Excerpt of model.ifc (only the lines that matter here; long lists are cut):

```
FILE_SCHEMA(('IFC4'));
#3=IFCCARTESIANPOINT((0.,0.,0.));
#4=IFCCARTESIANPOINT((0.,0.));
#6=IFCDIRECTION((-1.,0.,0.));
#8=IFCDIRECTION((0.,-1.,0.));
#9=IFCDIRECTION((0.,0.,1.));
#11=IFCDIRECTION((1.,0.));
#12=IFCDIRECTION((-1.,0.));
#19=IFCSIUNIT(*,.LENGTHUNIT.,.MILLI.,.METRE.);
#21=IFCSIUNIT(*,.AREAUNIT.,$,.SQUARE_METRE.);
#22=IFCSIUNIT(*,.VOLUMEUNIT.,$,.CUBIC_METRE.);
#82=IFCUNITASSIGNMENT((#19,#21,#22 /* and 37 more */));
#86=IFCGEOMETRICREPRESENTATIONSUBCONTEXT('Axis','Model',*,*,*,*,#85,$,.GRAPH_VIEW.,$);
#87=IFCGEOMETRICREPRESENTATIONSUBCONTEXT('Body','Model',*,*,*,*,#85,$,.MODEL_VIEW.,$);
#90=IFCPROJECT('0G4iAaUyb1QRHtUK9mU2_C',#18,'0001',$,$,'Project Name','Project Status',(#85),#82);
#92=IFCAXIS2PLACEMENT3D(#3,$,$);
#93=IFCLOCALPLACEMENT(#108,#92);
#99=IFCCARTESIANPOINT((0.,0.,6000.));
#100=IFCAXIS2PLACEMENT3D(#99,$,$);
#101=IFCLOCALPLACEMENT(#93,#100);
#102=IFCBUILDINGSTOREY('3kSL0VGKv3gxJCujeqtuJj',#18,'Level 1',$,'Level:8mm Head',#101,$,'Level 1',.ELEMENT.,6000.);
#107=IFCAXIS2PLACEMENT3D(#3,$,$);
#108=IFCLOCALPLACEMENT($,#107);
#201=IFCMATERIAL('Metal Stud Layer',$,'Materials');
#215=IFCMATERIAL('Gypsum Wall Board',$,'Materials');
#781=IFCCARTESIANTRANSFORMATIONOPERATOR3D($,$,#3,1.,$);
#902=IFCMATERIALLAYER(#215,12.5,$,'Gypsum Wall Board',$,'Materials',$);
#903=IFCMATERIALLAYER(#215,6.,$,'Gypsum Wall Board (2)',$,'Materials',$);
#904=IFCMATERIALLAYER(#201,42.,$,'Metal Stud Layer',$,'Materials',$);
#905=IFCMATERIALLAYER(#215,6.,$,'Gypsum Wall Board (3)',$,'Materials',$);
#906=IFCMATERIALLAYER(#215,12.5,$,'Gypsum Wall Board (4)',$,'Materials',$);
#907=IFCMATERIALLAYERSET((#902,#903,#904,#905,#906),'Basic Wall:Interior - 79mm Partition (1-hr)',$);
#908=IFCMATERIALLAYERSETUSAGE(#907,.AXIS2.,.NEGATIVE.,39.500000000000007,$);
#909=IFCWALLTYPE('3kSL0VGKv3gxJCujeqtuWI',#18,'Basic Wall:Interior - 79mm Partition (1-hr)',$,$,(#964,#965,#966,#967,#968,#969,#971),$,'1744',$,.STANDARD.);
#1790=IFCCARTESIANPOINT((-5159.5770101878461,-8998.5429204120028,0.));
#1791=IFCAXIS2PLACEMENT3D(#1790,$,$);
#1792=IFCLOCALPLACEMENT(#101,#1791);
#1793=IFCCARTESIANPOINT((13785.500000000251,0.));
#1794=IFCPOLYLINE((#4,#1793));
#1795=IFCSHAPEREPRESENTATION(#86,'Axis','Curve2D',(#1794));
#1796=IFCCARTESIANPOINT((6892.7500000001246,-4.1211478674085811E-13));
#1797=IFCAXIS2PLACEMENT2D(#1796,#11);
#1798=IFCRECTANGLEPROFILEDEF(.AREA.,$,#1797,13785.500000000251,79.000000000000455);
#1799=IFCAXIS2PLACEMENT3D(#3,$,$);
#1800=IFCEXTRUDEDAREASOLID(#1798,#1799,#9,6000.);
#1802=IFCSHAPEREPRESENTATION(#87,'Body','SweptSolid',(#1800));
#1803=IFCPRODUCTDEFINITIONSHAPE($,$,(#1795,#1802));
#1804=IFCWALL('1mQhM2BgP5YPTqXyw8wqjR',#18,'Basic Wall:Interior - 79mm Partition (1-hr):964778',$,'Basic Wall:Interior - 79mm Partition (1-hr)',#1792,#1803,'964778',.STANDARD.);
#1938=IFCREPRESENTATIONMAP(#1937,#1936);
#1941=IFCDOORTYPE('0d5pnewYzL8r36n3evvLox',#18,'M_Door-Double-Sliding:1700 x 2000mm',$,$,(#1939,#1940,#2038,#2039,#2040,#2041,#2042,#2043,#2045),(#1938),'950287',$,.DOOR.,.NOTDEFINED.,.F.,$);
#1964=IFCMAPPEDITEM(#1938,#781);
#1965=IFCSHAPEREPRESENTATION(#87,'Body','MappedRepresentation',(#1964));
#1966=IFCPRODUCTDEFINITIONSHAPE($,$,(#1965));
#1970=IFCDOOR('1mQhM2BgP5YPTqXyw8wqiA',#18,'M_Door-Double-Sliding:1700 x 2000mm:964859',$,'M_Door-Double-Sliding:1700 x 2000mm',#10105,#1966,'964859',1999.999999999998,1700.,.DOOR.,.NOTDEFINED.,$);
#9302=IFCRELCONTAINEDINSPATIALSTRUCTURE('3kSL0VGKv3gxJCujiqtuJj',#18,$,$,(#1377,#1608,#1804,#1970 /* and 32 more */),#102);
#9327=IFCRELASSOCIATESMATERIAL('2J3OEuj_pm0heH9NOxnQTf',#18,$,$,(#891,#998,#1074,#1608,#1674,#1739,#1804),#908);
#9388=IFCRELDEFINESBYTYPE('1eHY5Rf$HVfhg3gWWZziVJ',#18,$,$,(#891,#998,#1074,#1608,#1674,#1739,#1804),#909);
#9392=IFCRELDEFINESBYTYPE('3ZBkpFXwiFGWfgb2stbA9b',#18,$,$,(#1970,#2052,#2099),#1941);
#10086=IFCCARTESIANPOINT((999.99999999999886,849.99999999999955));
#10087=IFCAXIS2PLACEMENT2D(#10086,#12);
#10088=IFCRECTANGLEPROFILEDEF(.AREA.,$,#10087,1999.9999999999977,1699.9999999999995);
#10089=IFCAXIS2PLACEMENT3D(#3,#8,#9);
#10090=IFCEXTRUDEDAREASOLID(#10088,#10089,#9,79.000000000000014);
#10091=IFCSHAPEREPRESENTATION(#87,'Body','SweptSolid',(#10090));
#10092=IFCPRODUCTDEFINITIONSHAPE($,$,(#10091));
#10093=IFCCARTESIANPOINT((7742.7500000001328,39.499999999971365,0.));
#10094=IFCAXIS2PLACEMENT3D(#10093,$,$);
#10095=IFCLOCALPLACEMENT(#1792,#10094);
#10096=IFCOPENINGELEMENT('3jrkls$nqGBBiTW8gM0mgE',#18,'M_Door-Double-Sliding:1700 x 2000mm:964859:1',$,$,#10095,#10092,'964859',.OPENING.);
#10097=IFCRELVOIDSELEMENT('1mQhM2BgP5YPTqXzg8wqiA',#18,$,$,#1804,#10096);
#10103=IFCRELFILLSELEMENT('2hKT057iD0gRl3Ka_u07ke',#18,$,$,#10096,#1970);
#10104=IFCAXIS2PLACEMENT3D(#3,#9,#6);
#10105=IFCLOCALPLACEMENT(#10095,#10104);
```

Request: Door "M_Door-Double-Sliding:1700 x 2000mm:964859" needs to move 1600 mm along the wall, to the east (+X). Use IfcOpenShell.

```python
import ifcopenshell
import ifcopenshell.api.geometry
import ifcopenshell.util.placement
import ifcopenshell.util.unit

model = ifcopenshell.open("model.ifc")
unit_scale = ifcopenshell.util.unit.calculate_unit_scale(model)

door = model.by_id(1970)
opening = door.FillsVoids[0].RelatingOpeningElement
wall = opening.VoidsElements[0].RelatingBuildingElement

wall_matrix = ifcopenshell.util.placement.get_local_placement(wall.ObjectPlacement)
shift = wall_matrix[:3, 0] * 1.6 / unit_scale
before = ifcopenshell.util.placement.get_local_placement(door.ObjectPlacement)[:3, 3].copy()

# The door is placed relative to its opening, so it follows when the opening moves.
matrix = ifcopenshell.util.placement.get_local_placement(opening.ObjectPlacement)
matrix[:3, 3] += shift
ifcopenshell.api.geometry.edit_object_placement(
    model, product=opening, matrix=matrix, is_si=False, should_transform_children=True
)

after = ifcopenshell.util.placement.get_local_placement(door.ObjectPlacement)[:3, 3]
print("door moved by", (after - before).round(3) + 0.0)

model.write("model_edited.ifc")
```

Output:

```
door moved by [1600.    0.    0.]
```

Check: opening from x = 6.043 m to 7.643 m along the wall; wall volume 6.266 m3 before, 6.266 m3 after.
